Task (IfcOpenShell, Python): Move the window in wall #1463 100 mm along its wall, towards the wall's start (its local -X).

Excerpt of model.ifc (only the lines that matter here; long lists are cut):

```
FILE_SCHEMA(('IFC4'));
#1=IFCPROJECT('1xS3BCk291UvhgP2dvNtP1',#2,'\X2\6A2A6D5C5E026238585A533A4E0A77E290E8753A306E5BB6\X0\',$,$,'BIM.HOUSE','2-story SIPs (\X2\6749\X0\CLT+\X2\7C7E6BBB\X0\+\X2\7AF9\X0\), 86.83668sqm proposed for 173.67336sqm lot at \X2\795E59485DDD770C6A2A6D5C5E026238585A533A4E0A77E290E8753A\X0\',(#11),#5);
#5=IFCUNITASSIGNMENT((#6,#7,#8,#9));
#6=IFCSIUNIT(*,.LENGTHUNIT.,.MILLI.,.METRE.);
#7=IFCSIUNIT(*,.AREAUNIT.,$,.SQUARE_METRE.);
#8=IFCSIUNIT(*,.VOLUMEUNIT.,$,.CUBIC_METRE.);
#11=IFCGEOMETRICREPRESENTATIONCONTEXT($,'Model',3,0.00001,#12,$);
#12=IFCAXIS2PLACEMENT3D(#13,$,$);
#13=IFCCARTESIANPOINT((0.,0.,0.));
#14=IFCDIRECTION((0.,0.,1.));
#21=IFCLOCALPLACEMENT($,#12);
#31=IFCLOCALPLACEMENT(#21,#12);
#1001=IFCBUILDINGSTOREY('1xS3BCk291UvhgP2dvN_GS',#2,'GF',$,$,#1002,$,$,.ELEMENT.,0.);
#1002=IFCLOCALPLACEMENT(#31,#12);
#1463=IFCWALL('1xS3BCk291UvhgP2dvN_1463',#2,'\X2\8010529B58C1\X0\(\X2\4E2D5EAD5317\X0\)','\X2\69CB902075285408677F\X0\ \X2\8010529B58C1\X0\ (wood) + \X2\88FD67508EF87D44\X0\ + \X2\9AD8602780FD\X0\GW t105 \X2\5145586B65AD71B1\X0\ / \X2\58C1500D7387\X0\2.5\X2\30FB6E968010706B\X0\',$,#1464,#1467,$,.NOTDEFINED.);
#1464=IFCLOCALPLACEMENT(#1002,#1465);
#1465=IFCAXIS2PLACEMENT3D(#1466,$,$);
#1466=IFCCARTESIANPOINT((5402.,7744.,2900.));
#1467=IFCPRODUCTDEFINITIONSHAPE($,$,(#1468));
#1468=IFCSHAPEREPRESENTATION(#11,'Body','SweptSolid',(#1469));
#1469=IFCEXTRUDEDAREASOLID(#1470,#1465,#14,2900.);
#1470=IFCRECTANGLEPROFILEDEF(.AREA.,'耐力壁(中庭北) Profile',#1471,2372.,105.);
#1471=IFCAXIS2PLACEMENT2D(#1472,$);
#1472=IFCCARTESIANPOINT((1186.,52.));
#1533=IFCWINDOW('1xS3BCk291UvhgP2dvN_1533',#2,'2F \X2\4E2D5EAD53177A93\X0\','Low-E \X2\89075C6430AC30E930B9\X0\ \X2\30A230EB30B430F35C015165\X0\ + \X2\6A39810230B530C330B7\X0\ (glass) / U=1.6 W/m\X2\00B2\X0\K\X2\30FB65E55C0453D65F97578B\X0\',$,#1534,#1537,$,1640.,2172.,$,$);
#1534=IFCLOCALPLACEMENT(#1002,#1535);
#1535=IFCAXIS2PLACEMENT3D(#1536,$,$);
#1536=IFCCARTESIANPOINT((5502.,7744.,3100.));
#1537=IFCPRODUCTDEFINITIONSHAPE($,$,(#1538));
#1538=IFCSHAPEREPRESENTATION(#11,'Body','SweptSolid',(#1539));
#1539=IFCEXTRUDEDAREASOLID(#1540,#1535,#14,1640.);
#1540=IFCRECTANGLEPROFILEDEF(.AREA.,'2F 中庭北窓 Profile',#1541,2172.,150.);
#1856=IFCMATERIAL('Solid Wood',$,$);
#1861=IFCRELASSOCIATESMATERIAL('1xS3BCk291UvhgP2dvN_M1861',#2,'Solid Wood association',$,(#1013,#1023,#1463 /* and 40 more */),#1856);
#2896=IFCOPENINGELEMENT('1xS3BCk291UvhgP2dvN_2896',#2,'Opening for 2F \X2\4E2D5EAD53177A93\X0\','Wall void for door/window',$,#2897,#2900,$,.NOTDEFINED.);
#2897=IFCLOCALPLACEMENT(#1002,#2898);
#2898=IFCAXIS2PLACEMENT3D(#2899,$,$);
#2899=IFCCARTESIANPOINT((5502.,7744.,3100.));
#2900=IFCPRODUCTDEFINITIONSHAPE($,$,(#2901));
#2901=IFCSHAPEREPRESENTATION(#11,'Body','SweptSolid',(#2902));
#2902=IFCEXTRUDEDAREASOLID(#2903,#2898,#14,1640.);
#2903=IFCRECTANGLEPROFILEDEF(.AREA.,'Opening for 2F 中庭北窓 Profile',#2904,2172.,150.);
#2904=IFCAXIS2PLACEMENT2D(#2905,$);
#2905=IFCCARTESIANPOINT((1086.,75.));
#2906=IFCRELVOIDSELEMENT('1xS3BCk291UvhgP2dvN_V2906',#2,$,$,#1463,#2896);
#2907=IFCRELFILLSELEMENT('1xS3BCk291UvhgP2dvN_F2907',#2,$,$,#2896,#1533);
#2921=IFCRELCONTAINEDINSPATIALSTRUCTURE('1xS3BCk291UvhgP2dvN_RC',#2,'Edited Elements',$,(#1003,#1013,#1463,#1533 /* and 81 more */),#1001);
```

```python
import ifcopenshell
import ifcopenshell.api.geometry
import ifcopenshell.util.placement

model = ifcopenshell.open("model.ifc")

window = model.by_guid("1xS3BCk291UvhgP2dvN_1533")
opening = window.FillsVoids[0].RelatingOpeningElement
wall = opening.VoidsElements[0].RelatingBuildingElement

wall_matrix = ifcopenshell.util.placement.get_local_placement(wall.ObjectPlacement)
shift = wall_matrix[:3, 0] * -100.0
before = ifcopenshell.util.placement.get_local_placement(window.ObjectPlacement)[:3, 3].copy()

# The window is not placed relative to its opening, so move both.
for product in (opening, window):
    matrix = ifcopenshell.util.placement.get_local_placement(product.ObjectPlacement)
    matrix[:3, 3] += shift
    ifcopenshell.api.geometry.edit_object_placement(model, product=product, matrix=matrix, is_si=False)

after = ifcopenshell.util.placement.get_local_placement(window.ObjectPlacement)[:3, 3]
print("window moved by", (after - before).round(3) + 0.0)

model.write("model_rev.ifc")
```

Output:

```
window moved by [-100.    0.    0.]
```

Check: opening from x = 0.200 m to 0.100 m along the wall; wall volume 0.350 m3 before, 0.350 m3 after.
